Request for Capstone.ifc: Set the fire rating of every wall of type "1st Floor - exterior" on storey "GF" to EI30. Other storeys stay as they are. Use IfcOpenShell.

First a look at what the model holds.

```python
import ifcopenshell
import ifcopenshell.util.element

model = ifcopenshell.open("Capstone.ifc")
print(model.schema)
storey = next(s for s in model.by_type("IfcBuildingStorey") if s.Name == "GF")
walls = [e for e in ifcopenshell.util.element.get_decomposition(storey) if e.is_a("IfcWall")]
seen = {}
for e in walls:
    element_type = ifcopenshell.util.element.get_type(e)
    key = (element_type.Name if element_type != e and element_type else None, ifcopenshell.util.element.get_pset(e, "Pset_WallCommon", "FireRating"))
    seen[key] = seen.get(key, 0) + 1
for (name, value), count in sorted(seen.items(), key=str):
    print(count, "x", name, "|", value)
```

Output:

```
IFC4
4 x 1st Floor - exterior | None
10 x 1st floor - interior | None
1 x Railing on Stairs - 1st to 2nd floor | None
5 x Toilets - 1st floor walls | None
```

```python
import ifcopenshell
import ifcopenshell.api.pset
import ifcopenshell.util.element

model = ifcopenshell.open("Capstone.ifc")

storey = next(s for s in model.by_type("IfcBuildingStorey") if s.Name == "GF")
walls = [e for e in ifcopenshell.util.element.get_decomposition(storey) if e.is_a("IfcWall")]

count = 0
for e in walls:
    element_type = ifcopenshell.util.element.get_type(e)
    if element_type in (None, e) or element_type.Name != "1st Floor - exterior":
        continue
    # add_pset returns the element's existing set when there is one.
    pset = ifcopenshell.api.pset.add_pset(model, product=e, name="Pset_WallCommon")
    ifcopenshell.api.pset.edit_pset(model, pset=pset, properties={"FireRating": "EI30"})
    count += 1

print(count, "walls updated")

model.write("Capstone_rev.ifc")
```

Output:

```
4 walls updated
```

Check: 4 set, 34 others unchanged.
